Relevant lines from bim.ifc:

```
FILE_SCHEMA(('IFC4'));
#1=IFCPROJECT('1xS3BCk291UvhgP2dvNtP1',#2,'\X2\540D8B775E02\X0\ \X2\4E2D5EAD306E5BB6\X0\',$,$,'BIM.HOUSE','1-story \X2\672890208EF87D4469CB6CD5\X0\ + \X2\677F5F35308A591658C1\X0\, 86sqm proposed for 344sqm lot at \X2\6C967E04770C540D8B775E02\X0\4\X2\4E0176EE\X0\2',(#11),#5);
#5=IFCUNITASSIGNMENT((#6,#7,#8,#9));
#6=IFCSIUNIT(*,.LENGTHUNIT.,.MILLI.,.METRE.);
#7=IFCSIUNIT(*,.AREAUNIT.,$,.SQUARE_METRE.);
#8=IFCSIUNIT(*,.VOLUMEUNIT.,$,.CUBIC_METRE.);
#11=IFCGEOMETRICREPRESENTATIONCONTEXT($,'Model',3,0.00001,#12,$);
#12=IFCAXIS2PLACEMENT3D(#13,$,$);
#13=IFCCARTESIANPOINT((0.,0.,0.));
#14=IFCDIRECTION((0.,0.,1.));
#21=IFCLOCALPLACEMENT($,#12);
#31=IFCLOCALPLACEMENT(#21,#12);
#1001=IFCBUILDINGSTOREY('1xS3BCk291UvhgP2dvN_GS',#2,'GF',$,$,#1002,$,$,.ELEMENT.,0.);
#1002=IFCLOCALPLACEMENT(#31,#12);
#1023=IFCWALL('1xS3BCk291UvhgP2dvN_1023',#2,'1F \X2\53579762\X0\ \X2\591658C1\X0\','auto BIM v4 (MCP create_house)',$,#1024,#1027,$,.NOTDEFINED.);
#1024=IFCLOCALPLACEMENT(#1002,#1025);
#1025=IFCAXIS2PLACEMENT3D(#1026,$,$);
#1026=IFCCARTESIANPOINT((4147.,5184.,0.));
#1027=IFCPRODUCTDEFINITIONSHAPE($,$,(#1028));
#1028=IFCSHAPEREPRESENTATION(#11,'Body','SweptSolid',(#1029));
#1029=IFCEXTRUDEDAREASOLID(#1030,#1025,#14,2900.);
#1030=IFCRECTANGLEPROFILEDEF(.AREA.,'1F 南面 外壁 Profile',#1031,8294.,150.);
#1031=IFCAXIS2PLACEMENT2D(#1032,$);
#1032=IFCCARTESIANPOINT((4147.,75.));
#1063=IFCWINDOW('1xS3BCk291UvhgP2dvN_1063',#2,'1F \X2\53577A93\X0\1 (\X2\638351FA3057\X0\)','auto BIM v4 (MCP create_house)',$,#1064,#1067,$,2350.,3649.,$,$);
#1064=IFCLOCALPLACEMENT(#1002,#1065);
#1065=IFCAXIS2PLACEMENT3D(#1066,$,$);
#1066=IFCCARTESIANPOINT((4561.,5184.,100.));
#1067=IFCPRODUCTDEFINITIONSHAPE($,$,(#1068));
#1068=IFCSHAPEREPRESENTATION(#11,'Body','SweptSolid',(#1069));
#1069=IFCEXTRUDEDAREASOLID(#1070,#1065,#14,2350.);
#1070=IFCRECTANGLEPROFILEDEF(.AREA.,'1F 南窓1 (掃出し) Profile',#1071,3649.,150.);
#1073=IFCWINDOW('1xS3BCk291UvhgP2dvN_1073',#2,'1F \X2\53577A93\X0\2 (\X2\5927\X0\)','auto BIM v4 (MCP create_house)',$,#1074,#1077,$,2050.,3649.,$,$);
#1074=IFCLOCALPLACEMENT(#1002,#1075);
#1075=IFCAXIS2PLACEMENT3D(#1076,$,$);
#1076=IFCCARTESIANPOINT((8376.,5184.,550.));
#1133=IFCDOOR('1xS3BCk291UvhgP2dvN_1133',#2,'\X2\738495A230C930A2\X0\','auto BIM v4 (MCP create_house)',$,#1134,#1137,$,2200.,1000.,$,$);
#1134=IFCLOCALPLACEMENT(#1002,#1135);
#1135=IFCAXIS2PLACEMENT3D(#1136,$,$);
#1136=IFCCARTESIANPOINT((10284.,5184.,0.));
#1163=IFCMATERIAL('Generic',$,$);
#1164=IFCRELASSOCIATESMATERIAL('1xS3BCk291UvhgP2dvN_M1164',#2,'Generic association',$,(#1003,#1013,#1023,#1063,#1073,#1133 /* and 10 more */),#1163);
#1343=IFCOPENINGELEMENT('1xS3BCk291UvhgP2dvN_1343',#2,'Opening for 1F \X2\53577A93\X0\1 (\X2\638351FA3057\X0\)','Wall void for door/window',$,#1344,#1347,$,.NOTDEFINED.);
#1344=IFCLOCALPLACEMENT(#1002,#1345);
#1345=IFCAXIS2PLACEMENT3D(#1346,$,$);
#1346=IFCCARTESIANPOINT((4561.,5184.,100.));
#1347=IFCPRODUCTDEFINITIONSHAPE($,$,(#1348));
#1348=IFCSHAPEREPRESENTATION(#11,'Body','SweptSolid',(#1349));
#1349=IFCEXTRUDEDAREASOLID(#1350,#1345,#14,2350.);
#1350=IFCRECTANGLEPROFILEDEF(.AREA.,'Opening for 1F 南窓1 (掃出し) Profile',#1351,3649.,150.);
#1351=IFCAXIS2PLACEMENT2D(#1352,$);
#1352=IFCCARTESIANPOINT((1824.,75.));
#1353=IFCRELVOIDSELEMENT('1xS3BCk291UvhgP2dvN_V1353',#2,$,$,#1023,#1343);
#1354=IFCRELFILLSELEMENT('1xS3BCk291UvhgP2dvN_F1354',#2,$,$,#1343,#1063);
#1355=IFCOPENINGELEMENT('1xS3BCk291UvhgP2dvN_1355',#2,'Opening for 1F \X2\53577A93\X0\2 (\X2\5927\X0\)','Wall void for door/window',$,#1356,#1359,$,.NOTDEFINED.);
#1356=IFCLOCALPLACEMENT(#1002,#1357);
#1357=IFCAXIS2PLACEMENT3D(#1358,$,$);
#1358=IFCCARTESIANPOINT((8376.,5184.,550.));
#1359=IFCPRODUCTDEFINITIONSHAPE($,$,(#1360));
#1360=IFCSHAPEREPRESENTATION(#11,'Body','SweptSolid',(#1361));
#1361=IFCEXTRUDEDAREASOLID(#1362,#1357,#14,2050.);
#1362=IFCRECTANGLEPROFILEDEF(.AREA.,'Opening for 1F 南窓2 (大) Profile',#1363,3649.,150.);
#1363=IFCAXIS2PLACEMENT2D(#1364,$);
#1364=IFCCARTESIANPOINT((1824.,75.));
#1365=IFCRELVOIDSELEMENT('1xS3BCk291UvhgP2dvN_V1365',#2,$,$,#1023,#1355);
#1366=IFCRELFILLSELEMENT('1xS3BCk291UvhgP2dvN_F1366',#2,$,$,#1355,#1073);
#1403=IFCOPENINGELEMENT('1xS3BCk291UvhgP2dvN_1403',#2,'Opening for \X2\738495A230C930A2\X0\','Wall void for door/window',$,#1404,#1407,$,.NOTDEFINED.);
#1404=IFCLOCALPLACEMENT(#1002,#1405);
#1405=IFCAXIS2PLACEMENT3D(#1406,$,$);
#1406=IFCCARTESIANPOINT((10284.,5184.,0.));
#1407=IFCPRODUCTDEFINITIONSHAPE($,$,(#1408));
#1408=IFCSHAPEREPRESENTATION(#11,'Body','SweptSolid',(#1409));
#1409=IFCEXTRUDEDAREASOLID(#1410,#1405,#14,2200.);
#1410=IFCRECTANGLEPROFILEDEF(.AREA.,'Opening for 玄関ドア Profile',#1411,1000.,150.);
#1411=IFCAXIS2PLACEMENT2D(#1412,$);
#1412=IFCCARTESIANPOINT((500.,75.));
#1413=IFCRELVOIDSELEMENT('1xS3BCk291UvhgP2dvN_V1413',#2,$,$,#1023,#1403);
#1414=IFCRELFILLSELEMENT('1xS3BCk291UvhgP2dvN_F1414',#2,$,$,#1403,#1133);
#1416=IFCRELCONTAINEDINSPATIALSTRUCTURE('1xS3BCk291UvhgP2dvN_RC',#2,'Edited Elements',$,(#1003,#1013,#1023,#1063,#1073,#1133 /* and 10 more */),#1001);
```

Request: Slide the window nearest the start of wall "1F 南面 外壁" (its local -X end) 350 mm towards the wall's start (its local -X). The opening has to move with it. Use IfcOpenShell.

```python
import ifcopenshell
import ifcopenshell.api.geometry
import ifcopenshell.util.placement

model = ifcopenshell.open("bim.ifc")

window = model.by_id(1063)
opening = window.FillsVoids[0].RelatingOpeningElement
wall = opening.VoidsElements[0].RelatingBuildingElement

wall_matrix = ifcopenshell.util.placement.get_local_placement(wall.ObjectPlacement)
shift = wall_matrix[:3, 0] * -350.0
before = ifcopenshell.util.placement.get_local_placement(window.ObjectPlacement)[:3, 3].copy()

# The window is not placed relative to its opening, so move both.
for product in (opening, window):
    matrix = ifcopenshell.util.placement.get_local_placement(product.ObjectPlacement)
    matrix[:3, 3] += shift
    ifcopenshell.api.geometry.edit_object_placement(model, product=product, matrix=matrix, is_si=False)

after = ifcopenshell.util.placement.get_local_placement(window.ObjectPlacement)[:3, 3]
print("window moved by", (after - before).round(3) + 0.0)

model.write("bim_v2.ifc")
```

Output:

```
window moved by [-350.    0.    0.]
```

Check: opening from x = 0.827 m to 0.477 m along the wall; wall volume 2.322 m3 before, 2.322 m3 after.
